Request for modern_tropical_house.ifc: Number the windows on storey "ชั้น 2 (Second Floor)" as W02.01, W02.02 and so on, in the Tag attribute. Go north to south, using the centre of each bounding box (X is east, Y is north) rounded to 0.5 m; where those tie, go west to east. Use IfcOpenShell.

First a look at what the model holds.

```python
import ifcopenshell
import ifcopenshell.util.element
import ifcopenshell.util.placement

model = ifcopenshell.open("modern_tropical_house.ifc")
print(model.schema)
storey = next(s for s in model.by_type("IfcBuildingStorey") if s.Name == "ชั้น 2 (Second Floor)")
windows = [e for e in ifcopenshell.util.element.get_decomposition(storey) if e.is_a("IfcWindow")]
for e in sorted(windows, key=lambda e: e.id()):
    origin = ifcopenshell.util.placement.get_local_placement(e.ObjectPlacement)[:3, 3]
    print(e.id(), e.Tag, e.Name, origin.round(2) + 0.0, sep=" | ")
```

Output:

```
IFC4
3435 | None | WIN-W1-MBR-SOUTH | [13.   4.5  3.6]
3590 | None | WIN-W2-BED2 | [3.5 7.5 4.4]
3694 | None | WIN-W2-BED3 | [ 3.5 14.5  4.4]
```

```python
import ifcopenshell
import ifcopenshell.geom
import ifcopenshell.util.element
import ifcopenshell.util.shape

model = ifcopenshell.open("modern_tropical_house.ifc")
settings = ifcopenshell.geom.settings()
settings.set("use-world-coords", True)


def centre(element):
    shape = ifcopenshell.geom.create_shape(settings, element)
    return ifcopenshell.util.shape.get_bbox_centroid(shape.geometry)


storey = next(s for s in model.by_type("IfcBuildingStorey") if s.Name == "ชั้น 2 (Second Floor)")
windows = [e for e in ifcopenshell.util.element.get_decomposition(storey) if e.is_a("IfcWindow")]

# Insertion points can sit at a corner or the storey origin, so sort by the geometry (in metres).
centres = {e: centre(e) for e in windows}
windows.sort(key=lambda e: (-round(centres[e][1] / 0.5), centres[e][0]))

for i, e in enumerate(windows, start=1):
    number = f"W02.{i:02d}"
    e.Tag = number
    print(e.id(), number)

model.write("modern_tropical_house-out.ifc")
```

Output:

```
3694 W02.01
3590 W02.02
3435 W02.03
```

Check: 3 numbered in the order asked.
